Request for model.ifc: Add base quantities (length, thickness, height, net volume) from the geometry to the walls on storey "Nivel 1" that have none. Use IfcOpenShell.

First a look at what the model holds.

```python
import ifcopenshell
import ifcopenshell.util.element
import ifcopenshell.util.unit

model = ifcopenshell.open("model.ifc")
print(model.schema)
for unit_type in ("LENGTHUNIT", "AREAUNIT", "VOLUMEUNIT"):
    print(unit_type, ifcopenshell.util.unit.calculate_unit_scale(model, unit_type))
storey = next(s for s in model.by_type("IfcBuildingStorey") if s.Name == "Nivel 1")
walls = [e for e in ifcopenshell.util.element.get_decomposition(storey) if e.is_a("IfcWall")]
for e in sorted(walls, key=lambda e: e.id()):
    print(e.id(), e.is_a(), e.Name, list(ifcopenshell.util.element.get_psets(e, qtos_only=True)), sep=" | ")
```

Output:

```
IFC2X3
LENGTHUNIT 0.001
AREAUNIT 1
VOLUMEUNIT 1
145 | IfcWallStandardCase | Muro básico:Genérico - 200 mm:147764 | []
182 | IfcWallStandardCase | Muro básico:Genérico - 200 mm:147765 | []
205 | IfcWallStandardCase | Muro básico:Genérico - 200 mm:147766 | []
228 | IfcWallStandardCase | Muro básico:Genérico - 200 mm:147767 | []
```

```python
import ifcopenshell
import ifcopenshell.api.pset
import ifcopenshell.geom
import ifcopenshell.util.element
import ifcopenshell.util.shape
import ifcopenshell.util.unit

model = ifcopenshell.open("model.ifc")
unit_scale = ifcopenshell.util.unit.calculate_unit_scale(model)
volume_scale = ifcopenshell.util.unit.calculate_unit_scale(model, "VOLUMEUNIT")
settings = ifcopenshell.geom.settings()

storey = next(s for s in model.by_type("IfcBuildingStorey") if s.Name == "Nivel 1")
walls = [e for e in ifcopenshell.util.element.get_decomposition(storey) if e.is_a("IfcWall")]

for e in sorted(walls, key=lambda e: e.id()):
    if ifcopenshell.util.element.get_psets(e, qtos_only=True, should_inherit=False):
        continue
    # Geometry comes back in metres, in the element's own axes.
    shape = ifcopenshell.geom.create_shape(settings, e)
    values = {
        "Length": ifcopenshell.util.shape.get_x(shape.geometry) / unit_scale,
        "Width": ifcopenshell.util.shape.get_y(shape.geometry) / unit_scale,
        "Height": ifcopenshell.util.shape.get_z(shape.geometry) / unit_scale,
        "NetVolume": ifcopenshell.util.shape.get_volume(shape.geometry) / volume_scale,
    }
    qto = ifcopenshell.api.pset.add_qto(model, product=e, name="BaseQuantities")
    ifcopenshell.api.pset.edit_qto(model, qto=qto, properties=values)
    print(e.id(), {k: round(v, 3) for k, v in values.items()})

model.write("model_v2.ifc")
```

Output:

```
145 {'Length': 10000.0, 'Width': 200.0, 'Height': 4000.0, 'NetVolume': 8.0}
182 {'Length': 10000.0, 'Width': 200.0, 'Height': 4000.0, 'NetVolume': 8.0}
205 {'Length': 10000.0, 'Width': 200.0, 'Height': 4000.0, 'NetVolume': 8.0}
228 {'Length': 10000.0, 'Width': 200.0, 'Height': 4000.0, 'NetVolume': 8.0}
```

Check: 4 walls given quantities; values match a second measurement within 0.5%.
